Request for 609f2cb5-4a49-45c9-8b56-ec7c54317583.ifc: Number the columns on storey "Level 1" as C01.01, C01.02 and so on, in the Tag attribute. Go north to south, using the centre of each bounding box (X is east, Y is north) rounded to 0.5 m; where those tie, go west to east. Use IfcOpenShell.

First a look at what the model holds.

```python
import ifcopenshell
import ifcopenshell.util.element
import ifcopenshell.util.placement

model = ifcopenshell.open("609f2cb5-4a49-45c9-8b56-ec7c54317583.ifc")
print(model.schema)
storey = next(s for s in model.by_type("IfcBuildingStorey") if s.Name == "Level 1")
columns = [e for e in ifcopenshell.util.element.get_decomposition(storey) if e.is_a("IfcColumn")]
for e in sorted(columns, key=lambda e: e.id()):
    origin = ifcopenshell.util.placement.get_local_placement(e.ObjectPlacement)[:3, 3]
    print(e.id(), e.Tag, e.Name, origin.round(2) + 0.0, sep=" | ")
```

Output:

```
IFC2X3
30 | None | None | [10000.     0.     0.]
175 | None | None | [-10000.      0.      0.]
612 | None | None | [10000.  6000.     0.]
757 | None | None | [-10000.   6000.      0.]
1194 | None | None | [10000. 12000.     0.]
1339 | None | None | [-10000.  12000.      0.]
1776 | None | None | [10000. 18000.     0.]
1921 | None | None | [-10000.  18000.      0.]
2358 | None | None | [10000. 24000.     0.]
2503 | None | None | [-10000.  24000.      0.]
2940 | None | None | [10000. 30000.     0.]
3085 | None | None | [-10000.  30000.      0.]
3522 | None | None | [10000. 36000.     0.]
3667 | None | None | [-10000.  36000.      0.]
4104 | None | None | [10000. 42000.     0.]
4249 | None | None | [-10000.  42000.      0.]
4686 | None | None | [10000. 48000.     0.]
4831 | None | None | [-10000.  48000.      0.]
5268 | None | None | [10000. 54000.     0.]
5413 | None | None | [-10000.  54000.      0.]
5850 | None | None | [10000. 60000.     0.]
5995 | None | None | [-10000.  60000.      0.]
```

```python
import ifcopenshell
import ifcopenshell.geom
import ifcopenshell.util.element
import ifcopenshell.util.shape

model = ifcopenshell.open("609f2cb5-4a49-45c9-8b56-ec7c54317583.ifc")
settings = ifcopenshell.geom.settings()
settings.set("use-world-coords", True)


def centre(element):
    shape = ifcopenshell.geom.create_shape(settings, element)
    return ifcopenshell.util.shape.get_bbox_centroid(shape.geometry)


storey = next(s for s in model.by_type("IfcBuildingStorey") if s.Name == "Level 1")
columns = [e for e in ifcopenshell.util.element.get_decomposition(storey) if e.is_a("IfcColumn")]

# Insertion points can sit at a corner or the storey origin, so sort by the geometry (in metres).
centres = {e: centre(e) for e in columns}
columns.sort(key=lambda e: (-round(centres[e][1] / 0.5), centres[e][0]))

for i, e in enumerate(columns, start=1):
    number = f"C01.{i:02d}"
    e.Tag = number
    print(e.id(), number)

model.write("609f2cb5-4a49-45c9-8b56-ec7c54317583_v2.ifc")
```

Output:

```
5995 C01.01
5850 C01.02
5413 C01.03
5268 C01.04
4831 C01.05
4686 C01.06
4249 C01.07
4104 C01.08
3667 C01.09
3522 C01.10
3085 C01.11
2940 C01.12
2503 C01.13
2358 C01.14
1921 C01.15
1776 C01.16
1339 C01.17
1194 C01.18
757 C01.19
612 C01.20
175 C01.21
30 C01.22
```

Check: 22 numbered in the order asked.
